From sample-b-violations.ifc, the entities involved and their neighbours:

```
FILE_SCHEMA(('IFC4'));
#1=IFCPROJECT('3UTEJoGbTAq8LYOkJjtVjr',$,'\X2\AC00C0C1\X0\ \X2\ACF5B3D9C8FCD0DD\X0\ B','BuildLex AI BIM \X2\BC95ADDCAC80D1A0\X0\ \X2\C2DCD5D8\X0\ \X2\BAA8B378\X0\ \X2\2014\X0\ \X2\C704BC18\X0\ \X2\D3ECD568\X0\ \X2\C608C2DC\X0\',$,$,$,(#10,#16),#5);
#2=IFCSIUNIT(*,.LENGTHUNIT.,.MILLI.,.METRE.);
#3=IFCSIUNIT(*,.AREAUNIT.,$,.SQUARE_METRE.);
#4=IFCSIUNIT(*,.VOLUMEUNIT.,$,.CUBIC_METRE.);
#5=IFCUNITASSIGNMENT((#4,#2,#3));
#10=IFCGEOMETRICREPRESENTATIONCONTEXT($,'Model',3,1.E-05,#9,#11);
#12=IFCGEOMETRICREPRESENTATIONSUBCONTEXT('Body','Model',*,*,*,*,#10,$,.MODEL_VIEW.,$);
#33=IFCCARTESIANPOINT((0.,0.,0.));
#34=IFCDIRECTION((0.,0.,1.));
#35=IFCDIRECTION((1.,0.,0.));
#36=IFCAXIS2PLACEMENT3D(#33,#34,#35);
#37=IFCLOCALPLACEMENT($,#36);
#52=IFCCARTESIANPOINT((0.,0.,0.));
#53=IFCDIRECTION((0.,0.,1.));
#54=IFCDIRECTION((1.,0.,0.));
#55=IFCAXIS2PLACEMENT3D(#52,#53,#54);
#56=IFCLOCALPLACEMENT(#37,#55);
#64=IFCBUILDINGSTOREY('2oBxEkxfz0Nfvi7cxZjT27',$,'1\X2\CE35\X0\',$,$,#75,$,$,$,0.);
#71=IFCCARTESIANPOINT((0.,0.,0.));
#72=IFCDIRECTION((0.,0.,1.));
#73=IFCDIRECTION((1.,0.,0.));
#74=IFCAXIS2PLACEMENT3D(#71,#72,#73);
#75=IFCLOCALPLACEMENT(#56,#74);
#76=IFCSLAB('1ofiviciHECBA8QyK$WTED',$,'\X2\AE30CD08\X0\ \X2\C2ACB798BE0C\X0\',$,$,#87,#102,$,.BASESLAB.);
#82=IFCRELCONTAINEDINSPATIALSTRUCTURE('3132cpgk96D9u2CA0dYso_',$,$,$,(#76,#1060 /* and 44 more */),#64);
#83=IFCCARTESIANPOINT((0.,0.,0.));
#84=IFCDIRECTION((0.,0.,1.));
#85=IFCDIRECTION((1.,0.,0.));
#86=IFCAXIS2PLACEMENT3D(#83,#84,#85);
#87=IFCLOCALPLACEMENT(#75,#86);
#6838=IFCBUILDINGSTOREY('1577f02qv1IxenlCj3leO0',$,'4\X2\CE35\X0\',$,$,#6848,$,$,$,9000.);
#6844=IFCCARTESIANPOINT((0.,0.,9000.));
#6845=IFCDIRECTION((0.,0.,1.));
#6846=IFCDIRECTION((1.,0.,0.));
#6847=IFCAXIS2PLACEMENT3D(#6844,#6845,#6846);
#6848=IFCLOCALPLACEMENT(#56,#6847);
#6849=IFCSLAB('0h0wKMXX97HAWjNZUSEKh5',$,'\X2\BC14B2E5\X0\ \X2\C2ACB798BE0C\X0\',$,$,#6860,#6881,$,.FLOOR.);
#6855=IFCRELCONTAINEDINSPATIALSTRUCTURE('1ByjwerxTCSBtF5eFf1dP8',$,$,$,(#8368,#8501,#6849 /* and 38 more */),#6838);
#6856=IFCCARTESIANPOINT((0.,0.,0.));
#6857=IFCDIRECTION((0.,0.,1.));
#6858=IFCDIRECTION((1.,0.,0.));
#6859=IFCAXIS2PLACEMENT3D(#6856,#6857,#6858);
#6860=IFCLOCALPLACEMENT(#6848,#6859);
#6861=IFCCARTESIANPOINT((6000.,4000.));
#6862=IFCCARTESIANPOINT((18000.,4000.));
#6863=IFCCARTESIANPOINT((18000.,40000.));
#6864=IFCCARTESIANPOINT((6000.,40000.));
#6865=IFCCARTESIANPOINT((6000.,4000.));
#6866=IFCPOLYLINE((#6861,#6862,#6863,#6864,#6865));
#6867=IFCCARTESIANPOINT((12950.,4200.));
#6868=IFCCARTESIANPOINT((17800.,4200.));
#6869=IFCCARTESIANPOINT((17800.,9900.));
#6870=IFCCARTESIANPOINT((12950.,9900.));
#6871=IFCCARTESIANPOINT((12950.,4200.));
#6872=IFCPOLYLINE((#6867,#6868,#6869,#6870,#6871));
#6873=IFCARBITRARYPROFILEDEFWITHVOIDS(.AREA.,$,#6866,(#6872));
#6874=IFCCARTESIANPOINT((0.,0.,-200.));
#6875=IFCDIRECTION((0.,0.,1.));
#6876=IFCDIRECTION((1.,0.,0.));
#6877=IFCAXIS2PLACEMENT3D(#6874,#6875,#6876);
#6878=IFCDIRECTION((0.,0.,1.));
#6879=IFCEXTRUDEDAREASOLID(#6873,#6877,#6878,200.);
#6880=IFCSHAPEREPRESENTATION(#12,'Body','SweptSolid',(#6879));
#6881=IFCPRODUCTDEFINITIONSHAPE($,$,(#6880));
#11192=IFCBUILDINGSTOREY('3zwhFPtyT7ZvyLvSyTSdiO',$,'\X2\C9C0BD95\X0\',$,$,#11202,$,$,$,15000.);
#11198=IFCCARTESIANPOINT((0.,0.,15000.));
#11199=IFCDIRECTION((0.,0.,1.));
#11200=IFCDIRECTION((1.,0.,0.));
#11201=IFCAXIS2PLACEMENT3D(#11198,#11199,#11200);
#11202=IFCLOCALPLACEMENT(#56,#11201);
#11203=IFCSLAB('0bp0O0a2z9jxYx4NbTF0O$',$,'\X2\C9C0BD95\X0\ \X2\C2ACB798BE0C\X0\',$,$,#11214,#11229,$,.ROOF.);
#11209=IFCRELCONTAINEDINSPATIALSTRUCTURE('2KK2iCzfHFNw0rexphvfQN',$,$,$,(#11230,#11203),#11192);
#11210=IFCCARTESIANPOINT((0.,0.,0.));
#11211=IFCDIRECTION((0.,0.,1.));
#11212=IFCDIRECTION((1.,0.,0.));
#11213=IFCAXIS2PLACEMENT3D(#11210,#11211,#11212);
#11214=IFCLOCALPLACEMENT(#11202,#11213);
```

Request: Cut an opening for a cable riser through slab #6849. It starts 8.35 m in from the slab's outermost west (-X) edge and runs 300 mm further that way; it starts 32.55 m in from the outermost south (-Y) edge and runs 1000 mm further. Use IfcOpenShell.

```python
import numpy as np
import ifcopenshell
import ifcopenshell.api.feature
import ifcopenshell.api.geometry
import ifcopenshell.api.root
import ifcopenshell.geom
import ifcopenshell.util.placement
import ifcopenshell.util.representation
import ifcopenshell.util.shape
import ifcopenshell.util.unit

model = ifcopenshell.open("sample-b-violations.ifc")
unit_scale = ifcopenshell.util.unit.calculate_unit_scale(model)
settings = ifcopenshell.geom.settings()


def volume(element):
    """Net volume in cubic metres, openings subtracted."""
    shape = ifcopenshell.geom.create_shape(settings, element)
    return ifcopenshell.util.shape.get_volume(shape.geometry)


slab = model.by_guid("0h0wKMXX97HAWjNZUSEKh5")
before = volume(slab)

# Extent in the slab's own axes, in metres. The edges named are its -X and -Y sides.
slab_shape = ifcopenshell.geom.create_shape(settings, slab)
vertices = ifcopenshell.util.shape.get_vertices(slab_shape.geometry)
x_min, y_min, bottom = vertices.min(axis=0)
top = vertices[:, 2].max()

opening = ifcopenshell.api.root.create_entity(model, ifc_class="IfcOpeningElement", name="Cable riser opening", predefined_type="OPENING")
context = ifcopenshell.util.representation.get_context(model, "Model", "Body", "MODEL_VIEW")
width, depth = 0.3, 1
outline = [(0.0, 0.0), (width, 0.0), (width, depth), (0.0, depth), (0.0, 0.0)]
# Overshoot both faces by 50 mm so the cut is clean.
shape = ifcopenshell.api.geometry.add_slab_representation(
    model, context=context, depth=top - bottom + 0.1, polyline=outline
)
ifcopenshell.api.geometry.assign_representation(model, product=opening, representation=shape)

matrix = ifcopenshell.util.placement.get_local_placement(slab.ObjectPlacement)
matrix[:, 3] = matrix @ np.append(np.array([x_min + 8.35, y_min + 32.55, bottom - 0.05]) / unit_scale, 1.0)
ifcopenshell.api.geometry.edit_object_placement(model, product=opening, matrix=matrix, is_si=False)
ifcopenshell.api.feature.add_feature(model, feature=opening, element=slab)

after = volume(slab)

print(f"slab volume {before:.3f} -> {after:.3f} m3")

model.write("sample-b-violations_v2.ifc")
```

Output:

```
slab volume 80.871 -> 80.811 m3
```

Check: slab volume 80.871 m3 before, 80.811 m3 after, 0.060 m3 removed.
